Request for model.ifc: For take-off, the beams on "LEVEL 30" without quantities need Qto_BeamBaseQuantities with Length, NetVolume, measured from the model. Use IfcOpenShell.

First a look at what the model holds.

```python
import ifcopenshell
import ifcopenshell.util.element
import ifcopenshell.util.unit

model = ifcopenshell.open("model.ifc")
print(model.schema)
for unit_type in ("LENGTHUNIT", "AREAUNIT", "VOLUMEUNIT"):
    print(unit_type, ifcopenshell.util.unit.calculate_unit_scale(model, unit_type))
storey = next(s for s in model.by_type("IfcBuildingStorey") if s.Name == "LEVEL 30")
beams = [e for e in ifcopenshell.util.element.get_decomposition(storey) if e.is_a("IfcBeam")]
for e in sorted(beams, key=lambda e: e.id()):
    print(e.id(), e.is_a(), e.Name, list(ifcopenshell.util.element.get_psets(e, qtos_only=True)), sep=" | ")
```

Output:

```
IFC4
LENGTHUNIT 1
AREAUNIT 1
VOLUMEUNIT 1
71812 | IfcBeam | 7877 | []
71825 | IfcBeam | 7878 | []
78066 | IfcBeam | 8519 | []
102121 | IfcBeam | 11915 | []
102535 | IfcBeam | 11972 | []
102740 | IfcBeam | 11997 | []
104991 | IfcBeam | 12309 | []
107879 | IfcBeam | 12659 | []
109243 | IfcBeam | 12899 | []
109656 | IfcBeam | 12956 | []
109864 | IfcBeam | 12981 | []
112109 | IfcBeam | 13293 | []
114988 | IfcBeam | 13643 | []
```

```python
import ifcopenshell
import ifcopenshell.api.pset
import ifcopenshell.geom
import ifcopenshell.util.element
import ifcopenshell.util.shape
import ifcopenshell.util.unit

model = ifcopenshell.open("model.ifc")
unit_scale = ifcopenshell.util.unit.calculate_unit_scale(model)
volume_scale = ifcopenshell.util.unit.calculate_unit_scale(model, "VOLUMEUNIT")
settings = ifcopenshell.geom.settings()

storey = next(s for s in model.by_type("IfcBuildingStorey") if s.Name == "LEVEL 30")
beams = [e for e in ifcopenshell.util.element.get_decomposition(storey) if e.is_a("IfcBeam")]

for e in sorted(beams, key=lambda e: e.id()):
    if ifcopenshell.util.element.get_psets(e, qtos_only=True, should_inherit=False):
        continue
    # Geometry comes back in metres, in the element's own axes.
    shape = ifcopenshell.geom.create_shape(settings, e)
    values = {
        "Length": ifcopenshell.util.shape.get_max_xyz(shape.geometry) / unit_scale,
        "NetVolume": ifcopenshell.util.shape.get_volume(shape.geometry) / volume_scale,
    }
    qto = ifcopenshell.api.pset.add_qto(model, product=e, name="Qto_BeamBaseQuantities")
    ifcopenshell.api.pset.edit_qto(model, qto=qto, properties=values)
    print(e.id(), {k: round(v, 3) for k, v in values.items()})

model.write("model-out.ifc")
```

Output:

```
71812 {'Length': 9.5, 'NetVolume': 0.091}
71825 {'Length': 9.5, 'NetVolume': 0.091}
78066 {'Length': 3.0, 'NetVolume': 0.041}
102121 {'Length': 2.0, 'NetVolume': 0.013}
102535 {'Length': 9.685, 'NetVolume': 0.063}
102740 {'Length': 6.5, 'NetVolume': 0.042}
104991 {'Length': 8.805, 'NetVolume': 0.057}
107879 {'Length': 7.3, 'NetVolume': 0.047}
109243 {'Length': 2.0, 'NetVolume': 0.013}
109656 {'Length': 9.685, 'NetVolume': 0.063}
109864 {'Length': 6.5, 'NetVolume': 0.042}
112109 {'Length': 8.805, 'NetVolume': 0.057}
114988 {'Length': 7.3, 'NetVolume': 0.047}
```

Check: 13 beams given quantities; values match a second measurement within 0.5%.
